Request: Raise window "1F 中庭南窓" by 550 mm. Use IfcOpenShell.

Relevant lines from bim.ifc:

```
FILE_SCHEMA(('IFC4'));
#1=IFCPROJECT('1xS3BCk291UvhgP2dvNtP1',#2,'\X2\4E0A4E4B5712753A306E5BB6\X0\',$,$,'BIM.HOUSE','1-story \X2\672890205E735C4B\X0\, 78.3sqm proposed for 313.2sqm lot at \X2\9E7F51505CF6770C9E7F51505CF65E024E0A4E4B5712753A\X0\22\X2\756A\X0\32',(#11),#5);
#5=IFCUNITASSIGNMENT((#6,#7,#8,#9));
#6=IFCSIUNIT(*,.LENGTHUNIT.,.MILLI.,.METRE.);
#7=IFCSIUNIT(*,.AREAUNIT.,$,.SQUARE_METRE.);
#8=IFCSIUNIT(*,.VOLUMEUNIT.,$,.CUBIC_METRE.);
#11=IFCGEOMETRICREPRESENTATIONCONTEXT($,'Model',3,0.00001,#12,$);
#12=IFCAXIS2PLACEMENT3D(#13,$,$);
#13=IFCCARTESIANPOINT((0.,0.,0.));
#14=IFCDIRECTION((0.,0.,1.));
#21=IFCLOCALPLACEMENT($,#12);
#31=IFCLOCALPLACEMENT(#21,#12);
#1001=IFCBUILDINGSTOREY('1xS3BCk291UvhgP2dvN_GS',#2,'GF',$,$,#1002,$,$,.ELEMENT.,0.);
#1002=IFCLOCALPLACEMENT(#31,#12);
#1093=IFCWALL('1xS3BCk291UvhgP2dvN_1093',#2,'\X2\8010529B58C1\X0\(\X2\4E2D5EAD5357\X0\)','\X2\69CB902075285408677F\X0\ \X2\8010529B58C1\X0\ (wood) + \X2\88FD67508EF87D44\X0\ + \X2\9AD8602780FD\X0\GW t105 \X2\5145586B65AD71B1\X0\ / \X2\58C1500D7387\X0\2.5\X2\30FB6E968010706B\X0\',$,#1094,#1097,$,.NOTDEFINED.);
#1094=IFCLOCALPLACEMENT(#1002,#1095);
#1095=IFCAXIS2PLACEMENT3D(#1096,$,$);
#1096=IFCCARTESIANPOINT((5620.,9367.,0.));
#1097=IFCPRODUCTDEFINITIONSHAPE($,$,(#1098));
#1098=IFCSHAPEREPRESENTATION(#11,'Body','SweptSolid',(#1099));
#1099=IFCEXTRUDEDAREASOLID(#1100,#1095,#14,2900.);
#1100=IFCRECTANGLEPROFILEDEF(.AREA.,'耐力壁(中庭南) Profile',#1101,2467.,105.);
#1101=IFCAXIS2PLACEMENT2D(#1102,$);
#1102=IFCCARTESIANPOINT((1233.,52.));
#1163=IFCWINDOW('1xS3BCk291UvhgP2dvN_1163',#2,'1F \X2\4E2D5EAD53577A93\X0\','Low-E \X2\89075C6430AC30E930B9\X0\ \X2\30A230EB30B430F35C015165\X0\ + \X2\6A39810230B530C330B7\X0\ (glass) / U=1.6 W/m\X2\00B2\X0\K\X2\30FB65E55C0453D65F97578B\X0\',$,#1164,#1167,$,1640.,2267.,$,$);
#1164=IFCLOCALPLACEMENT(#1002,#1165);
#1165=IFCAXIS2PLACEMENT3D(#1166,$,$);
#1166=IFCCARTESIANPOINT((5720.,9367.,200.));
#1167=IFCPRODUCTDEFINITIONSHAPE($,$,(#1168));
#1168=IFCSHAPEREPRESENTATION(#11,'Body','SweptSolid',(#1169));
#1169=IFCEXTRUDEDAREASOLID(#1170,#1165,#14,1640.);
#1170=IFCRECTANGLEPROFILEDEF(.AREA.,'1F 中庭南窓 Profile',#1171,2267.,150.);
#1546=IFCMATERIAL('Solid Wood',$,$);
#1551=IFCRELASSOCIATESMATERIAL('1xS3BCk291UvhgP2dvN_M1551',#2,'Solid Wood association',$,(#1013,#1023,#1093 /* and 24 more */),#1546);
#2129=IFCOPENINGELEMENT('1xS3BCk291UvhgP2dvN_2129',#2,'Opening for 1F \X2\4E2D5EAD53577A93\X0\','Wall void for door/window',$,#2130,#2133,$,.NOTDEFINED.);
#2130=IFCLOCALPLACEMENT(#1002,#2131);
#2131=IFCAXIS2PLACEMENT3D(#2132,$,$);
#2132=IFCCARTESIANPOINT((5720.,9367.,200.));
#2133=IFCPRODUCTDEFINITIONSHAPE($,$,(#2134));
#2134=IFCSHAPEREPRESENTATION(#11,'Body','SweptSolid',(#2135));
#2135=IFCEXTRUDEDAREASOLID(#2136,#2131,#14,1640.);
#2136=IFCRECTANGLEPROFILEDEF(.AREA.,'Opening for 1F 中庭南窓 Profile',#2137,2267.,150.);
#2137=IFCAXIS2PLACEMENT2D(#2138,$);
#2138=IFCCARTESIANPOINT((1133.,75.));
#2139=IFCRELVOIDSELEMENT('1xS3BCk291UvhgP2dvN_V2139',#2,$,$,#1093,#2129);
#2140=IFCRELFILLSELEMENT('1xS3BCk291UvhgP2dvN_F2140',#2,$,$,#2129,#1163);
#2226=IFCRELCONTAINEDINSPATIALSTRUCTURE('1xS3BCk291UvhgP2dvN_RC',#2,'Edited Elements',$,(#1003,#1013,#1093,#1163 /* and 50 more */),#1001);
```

```python
import numpy as np
import ifcopenshell
import ifcopenshell.api.geometry
import ifcopenshell.util.placement
import ifcopenshell.util.unit

model = ifcopenshell.open("bim.ifc")
unit_scale = ifcopenshell.util.unit.calculate_unit_scale(model)

window = model.by_id(1163)
opening = window.FillsVoids[0].RelatingOpeningElement
dz = 0.55 / unit_scale

shift = np.array([0.0, 0.0, dz])
# The window is not placed relative to its opening, so move both.
for product in (opening, window):
    matrix = ifcopenshell.util.placement.get_local_placement(product.ObjectPlacement)
    matrix[:3, 3] += shift
    ifcopenshell.api.geometry.edit_object_placement(model, product=product, matrix=matrix, is_si=False)

print(f"moved by {dz * unit_scale:+.3f} m")

model.write("bim_rev.ifc")
```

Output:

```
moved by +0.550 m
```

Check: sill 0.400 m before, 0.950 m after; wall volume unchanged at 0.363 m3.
